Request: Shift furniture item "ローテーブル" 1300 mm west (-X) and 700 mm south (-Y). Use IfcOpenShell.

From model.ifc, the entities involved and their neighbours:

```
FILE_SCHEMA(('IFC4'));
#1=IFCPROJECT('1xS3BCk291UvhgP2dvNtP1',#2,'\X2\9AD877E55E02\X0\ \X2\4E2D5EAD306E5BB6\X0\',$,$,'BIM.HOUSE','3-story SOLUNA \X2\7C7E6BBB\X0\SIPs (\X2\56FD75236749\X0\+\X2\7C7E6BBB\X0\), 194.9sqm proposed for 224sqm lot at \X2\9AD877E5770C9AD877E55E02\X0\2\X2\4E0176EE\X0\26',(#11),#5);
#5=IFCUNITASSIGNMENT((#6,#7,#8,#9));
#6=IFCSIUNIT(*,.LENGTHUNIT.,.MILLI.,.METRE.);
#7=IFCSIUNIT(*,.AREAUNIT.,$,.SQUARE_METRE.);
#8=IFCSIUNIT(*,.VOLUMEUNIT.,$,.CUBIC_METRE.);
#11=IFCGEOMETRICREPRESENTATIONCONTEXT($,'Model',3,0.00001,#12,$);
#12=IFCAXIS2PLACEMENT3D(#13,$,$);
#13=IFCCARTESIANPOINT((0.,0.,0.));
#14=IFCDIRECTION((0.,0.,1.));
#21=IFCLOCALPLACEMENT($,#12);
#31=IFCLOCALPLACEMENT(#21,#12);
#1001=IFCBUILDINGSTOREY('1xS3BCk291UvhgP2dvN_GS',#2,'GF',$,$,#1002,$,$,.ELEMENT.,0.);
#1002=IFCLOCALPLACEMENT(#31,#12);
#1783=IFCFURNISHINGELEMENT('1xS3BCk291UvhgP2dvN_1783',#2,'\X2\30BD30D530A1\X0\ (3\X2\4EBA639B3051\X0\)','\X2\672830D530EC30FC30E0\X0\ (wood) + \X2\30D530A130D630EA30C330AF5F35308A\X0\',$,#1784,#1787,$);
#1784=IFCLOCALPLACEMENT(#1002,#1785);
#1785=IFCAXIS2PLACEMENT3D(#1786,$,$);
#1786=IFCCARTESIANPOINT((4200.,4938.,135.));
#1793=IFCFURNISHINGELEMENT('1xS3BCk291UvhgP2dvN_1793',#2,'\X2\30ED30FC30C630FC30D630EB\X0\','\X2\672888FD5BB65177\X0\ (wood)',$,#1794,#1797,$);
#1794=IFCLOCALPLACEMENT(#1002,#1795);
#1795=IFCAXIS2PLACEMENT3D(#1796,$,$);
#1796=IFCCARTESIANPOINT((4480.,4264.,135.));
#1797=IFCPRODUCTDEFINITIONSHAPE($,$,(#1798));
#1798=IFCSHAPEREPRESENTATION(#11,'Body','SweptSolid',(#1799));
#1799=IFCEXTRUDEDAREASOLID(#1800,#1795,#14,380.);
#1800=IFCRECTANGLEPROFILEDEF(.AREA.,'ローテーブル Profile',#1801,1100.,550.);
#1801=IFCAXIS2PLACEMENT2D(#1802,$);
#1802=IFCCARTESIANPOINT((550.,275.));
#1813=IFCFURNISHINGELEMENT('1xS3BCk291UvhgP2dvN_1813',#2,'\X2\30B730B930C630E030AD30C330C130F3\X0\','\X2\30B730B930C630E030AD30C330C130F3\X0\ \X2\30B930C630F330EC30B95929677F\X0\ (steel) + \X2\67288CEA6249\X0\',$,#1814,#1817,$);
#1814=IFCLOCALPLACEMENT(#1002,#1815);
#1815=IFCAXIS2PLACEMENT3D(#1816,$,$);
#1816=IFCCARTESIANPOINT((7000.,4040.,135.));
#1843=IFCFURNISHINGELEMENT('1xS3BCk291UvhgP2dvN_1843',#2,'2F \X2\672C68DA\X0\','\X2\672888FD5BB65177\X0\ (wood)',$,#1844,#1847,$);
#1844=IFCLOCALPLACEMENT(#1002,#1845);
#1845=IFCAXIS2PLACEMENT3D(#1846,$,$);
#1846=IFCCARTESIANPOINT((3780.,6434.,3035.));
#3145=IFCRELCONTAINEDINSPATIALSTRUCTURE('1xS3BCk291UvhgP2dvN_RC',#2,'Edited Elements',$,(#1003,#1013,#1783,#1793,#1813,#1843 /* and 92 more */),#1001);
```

```python
import ifcopenshell
import ifcopenshell.api.geometry
import ifcopenshell.util.placement
import ifcopenshell.util.unit

model = ifcopenshell.open("model.ifc")
unit_scale = ifcopenshell.util.unit.calculate_unit_scale(model)

item = model.by_guid("1xS3BCk291UvhgP2dvN_1793")
matrix = ifcopenshell.util.placement.get_local_placement(item.ObjectPlacement)
matrix[0, 3] -= 1.3 / unit_scale
matrix[1, 3] -= 0.7 / unit_scale
ifcopenshell.api.geometry.edit_object_placement(model, product=item, matrix=matrix, is_si=False)

print(ifcopenshell.util.placement.get_local_placement(item.ObjectPlacement).round(3) + 0.0)

model.write("model_v2.ifc")
```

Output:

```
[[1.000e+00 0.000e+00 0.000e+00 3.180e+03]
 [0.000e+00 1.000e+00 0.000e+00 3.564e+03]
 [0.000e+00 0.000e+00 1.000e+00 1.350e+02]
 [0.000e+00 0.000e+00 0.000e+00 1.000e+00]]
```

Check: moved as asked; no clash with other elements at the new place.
